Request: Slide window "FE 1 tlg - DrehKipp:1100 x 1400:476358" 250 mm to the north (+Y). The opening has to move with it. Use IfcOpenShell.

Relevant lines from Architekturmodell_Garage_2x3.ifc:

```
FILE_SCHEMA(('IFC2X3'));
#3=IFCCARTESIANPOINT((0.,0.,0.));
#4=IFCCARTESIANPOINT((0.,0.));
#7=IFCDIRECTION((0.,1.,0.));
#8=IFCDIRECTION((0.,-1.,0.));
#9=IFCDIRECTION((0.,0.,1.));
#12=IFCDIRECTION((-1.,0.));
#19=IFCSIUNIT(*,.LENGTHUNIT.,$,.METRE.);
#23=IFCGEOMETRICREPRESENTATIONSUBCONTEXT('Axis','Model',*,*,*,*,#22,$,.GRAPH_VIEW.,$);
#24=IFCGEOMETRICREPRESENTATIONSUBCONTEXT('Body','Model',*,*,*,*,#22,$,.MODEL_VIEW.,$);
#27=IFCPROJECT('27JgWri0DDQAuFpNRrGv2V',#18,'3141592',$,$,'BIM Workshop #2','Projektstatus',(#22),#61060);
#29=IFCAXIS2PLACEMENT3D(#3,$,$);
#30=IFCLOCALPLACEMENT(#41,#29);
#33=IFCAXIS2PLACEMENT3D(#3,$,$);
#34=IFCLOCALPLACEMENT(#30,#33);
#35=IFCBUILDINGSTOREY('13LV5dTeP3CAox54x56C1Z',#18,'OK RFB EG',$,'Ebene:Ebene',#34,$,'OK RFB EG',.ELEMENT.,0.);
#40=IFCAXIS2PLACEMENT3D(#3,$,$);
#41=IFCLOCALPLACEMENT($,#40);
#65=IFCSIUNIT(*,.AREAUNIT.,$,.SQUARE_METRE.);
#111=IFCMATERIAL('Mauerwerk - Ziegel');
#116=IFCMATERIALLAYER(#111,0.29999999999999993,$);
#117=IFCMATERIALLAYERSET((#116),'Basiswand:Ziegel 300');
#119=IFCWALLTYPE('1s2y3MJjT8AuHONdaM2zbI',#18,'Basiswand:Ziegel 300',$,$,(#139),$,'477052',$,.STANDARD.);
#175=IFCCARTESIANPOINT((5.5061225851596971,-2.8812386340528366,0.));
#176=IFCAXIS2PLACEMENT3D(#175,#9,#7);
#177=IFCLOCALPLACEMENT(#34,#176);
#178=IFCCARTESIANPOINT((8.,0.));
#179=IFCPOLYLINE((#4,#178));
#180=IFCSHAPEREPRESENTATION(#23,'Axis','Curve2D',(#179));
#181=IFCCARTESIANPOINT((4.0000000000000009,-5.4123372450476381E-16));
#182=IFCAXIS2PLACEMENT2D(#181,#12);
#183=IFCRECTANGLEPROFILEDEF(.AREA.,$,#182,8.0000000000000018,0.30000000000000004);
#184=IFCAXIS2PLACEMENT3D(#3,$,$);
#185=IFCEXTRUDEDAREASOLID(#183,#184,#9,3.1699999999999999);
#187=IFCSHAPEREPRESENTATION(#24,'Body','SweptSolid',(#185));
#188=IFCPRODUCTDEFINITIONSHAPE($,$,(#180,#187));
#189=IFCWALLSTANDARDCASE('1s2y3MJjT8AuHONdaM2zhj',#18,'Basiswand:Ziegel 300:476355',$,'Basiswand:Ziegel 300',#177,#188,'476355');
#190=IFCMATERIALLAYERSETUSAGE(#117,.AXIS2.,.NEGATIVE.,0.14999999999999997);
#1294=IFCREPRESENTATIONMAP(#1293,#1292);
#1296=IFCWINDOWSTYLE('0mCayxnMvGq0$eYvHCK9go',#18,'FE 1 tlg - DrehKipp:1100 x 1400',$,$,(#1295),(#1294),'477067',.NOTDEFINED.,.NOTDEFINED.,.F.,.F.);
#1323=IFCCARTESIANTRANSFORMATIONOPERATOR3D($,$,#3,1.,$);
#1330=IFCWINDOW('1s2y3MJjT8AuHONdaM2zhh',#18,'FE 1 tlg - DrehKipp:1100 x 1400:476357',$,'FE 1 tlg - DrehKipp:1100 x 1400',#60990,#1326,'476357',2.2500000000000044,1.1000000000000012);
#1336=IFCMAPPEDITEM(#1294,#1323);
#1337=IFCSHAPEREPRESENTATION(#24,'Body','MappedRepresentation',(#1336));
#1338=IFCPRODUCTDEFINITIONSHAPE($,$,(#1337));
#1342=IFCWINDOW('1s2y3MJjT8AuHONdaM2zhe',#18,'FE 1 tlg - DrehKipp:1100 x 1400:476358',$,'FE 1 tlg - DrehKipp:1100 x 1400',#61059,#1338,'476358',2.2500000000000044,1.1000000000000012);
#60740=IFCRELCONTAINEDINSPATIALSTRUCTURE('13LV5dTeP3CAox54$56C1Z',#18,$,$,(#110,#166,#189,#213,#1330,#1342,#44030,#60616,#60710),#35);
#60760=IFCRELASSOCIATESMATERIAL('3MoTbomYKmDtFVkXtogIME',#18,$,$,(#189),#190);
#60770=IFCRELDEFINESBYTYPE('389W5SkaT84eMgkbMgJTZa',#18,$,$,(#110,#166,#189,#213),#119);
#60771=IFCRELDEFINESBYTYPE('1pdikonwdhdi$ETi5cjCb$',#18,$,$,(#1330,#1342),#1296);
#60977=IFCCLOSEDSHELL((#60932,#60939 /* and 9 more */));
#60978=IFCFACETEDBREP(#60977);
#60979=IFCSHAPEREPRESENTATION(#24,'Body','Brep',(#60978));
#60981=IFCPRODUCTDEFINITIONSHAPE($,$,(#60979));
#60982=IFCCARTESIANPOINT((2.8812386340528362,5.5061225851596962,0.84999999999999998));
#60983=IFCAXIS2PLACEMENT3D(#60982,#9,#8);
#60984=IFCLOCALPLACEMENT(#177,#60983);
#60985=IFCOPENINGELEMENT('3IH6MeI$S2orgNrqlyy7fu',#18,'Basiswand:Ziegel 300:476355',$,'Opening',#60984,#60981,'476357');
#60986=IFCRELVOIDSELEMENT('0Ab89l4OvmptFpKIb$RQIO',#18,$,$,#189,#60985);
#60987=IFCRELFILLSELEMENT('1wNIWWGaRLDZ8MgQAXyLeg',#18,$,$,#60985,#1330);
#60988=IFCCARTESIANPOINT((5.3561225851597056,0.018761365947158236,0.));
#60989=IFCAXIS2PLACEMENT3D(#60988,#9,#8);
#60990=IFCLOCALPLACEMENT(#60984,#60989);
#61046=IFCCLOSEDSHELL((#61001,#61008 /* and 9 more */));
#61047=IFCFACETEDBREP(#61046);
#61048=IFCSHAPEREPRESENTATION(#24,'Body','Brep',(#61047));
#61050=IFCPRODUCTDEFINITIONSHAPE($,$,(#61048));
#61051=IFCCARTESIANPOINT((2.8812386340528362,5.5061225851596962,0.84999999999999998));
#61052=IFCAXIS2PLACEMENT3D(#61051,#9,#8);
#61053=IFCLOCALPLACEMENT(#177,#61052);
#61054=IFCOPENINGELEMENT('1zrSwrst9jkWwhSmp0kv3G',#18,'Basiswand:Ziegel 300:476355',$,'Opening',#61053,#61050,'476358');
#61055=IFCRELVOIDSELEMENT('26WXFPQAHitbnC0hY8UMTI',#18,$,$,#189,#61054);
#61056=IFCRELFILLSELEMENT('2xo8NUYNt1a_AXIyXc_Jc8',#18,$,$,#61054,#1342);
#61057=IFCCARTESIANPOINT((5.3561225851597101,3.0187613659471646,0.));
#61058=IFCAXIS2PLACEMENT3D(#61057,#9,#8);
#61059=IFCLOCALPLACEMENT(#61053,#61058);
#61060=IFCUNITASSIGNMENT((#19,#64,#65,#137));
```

```python
import ifcopenshell
import ifcopenshell.api.geometry
import ifcopenshell.util.placement
import ifcopenshell.util.unit

model = ifcopenshell.open("Architekturmodell_Garage_2x3.ifc")
unit_scale = ifcopenshell.util.unit.calculate_unit_scale(model)

window = model.by_guid("1s2y3MJjT8AuHONdaM2zhe")
opening = window.FillsVoids[0].RelatingOpeningElement
wall = opening.VoidsElements[0].RelatingBuildingElement

wall_matrix = ifcopenshell.util.placement.get_local_placement(wall.ObjectPlacement)
shift = wall_matrix[:3, 0] * 0.25 / unit_scale
before = ifcopenshell.util.placement.get_local_placement(window.ObjectPlacement)[:3, 3].copy()

# The window is placed relative to its opening, so it follows when the opening moves.
matrix = ifcopenshell.util.placement.get_local_placement(opening.ObjectPlacement)
matrix[:3, 3] += shift
ifcopenshell.api.geometry.edit_object_placement(
    model, product=opening, matrix=matrix, is_si=False, should_transform_children=True
)

after = ifcopenshell.util.placement.get_local_placement(window.ObjectPlacement)[:3, 3]
print("window moved by", (after - before).round(3) + 0.0)

model.write("Architekturmodell_Garage_2x3-out.ifc")
```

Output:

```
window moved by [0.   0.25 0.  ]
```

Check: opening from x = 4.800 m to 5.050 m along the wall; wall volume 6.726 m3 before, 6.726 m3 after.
